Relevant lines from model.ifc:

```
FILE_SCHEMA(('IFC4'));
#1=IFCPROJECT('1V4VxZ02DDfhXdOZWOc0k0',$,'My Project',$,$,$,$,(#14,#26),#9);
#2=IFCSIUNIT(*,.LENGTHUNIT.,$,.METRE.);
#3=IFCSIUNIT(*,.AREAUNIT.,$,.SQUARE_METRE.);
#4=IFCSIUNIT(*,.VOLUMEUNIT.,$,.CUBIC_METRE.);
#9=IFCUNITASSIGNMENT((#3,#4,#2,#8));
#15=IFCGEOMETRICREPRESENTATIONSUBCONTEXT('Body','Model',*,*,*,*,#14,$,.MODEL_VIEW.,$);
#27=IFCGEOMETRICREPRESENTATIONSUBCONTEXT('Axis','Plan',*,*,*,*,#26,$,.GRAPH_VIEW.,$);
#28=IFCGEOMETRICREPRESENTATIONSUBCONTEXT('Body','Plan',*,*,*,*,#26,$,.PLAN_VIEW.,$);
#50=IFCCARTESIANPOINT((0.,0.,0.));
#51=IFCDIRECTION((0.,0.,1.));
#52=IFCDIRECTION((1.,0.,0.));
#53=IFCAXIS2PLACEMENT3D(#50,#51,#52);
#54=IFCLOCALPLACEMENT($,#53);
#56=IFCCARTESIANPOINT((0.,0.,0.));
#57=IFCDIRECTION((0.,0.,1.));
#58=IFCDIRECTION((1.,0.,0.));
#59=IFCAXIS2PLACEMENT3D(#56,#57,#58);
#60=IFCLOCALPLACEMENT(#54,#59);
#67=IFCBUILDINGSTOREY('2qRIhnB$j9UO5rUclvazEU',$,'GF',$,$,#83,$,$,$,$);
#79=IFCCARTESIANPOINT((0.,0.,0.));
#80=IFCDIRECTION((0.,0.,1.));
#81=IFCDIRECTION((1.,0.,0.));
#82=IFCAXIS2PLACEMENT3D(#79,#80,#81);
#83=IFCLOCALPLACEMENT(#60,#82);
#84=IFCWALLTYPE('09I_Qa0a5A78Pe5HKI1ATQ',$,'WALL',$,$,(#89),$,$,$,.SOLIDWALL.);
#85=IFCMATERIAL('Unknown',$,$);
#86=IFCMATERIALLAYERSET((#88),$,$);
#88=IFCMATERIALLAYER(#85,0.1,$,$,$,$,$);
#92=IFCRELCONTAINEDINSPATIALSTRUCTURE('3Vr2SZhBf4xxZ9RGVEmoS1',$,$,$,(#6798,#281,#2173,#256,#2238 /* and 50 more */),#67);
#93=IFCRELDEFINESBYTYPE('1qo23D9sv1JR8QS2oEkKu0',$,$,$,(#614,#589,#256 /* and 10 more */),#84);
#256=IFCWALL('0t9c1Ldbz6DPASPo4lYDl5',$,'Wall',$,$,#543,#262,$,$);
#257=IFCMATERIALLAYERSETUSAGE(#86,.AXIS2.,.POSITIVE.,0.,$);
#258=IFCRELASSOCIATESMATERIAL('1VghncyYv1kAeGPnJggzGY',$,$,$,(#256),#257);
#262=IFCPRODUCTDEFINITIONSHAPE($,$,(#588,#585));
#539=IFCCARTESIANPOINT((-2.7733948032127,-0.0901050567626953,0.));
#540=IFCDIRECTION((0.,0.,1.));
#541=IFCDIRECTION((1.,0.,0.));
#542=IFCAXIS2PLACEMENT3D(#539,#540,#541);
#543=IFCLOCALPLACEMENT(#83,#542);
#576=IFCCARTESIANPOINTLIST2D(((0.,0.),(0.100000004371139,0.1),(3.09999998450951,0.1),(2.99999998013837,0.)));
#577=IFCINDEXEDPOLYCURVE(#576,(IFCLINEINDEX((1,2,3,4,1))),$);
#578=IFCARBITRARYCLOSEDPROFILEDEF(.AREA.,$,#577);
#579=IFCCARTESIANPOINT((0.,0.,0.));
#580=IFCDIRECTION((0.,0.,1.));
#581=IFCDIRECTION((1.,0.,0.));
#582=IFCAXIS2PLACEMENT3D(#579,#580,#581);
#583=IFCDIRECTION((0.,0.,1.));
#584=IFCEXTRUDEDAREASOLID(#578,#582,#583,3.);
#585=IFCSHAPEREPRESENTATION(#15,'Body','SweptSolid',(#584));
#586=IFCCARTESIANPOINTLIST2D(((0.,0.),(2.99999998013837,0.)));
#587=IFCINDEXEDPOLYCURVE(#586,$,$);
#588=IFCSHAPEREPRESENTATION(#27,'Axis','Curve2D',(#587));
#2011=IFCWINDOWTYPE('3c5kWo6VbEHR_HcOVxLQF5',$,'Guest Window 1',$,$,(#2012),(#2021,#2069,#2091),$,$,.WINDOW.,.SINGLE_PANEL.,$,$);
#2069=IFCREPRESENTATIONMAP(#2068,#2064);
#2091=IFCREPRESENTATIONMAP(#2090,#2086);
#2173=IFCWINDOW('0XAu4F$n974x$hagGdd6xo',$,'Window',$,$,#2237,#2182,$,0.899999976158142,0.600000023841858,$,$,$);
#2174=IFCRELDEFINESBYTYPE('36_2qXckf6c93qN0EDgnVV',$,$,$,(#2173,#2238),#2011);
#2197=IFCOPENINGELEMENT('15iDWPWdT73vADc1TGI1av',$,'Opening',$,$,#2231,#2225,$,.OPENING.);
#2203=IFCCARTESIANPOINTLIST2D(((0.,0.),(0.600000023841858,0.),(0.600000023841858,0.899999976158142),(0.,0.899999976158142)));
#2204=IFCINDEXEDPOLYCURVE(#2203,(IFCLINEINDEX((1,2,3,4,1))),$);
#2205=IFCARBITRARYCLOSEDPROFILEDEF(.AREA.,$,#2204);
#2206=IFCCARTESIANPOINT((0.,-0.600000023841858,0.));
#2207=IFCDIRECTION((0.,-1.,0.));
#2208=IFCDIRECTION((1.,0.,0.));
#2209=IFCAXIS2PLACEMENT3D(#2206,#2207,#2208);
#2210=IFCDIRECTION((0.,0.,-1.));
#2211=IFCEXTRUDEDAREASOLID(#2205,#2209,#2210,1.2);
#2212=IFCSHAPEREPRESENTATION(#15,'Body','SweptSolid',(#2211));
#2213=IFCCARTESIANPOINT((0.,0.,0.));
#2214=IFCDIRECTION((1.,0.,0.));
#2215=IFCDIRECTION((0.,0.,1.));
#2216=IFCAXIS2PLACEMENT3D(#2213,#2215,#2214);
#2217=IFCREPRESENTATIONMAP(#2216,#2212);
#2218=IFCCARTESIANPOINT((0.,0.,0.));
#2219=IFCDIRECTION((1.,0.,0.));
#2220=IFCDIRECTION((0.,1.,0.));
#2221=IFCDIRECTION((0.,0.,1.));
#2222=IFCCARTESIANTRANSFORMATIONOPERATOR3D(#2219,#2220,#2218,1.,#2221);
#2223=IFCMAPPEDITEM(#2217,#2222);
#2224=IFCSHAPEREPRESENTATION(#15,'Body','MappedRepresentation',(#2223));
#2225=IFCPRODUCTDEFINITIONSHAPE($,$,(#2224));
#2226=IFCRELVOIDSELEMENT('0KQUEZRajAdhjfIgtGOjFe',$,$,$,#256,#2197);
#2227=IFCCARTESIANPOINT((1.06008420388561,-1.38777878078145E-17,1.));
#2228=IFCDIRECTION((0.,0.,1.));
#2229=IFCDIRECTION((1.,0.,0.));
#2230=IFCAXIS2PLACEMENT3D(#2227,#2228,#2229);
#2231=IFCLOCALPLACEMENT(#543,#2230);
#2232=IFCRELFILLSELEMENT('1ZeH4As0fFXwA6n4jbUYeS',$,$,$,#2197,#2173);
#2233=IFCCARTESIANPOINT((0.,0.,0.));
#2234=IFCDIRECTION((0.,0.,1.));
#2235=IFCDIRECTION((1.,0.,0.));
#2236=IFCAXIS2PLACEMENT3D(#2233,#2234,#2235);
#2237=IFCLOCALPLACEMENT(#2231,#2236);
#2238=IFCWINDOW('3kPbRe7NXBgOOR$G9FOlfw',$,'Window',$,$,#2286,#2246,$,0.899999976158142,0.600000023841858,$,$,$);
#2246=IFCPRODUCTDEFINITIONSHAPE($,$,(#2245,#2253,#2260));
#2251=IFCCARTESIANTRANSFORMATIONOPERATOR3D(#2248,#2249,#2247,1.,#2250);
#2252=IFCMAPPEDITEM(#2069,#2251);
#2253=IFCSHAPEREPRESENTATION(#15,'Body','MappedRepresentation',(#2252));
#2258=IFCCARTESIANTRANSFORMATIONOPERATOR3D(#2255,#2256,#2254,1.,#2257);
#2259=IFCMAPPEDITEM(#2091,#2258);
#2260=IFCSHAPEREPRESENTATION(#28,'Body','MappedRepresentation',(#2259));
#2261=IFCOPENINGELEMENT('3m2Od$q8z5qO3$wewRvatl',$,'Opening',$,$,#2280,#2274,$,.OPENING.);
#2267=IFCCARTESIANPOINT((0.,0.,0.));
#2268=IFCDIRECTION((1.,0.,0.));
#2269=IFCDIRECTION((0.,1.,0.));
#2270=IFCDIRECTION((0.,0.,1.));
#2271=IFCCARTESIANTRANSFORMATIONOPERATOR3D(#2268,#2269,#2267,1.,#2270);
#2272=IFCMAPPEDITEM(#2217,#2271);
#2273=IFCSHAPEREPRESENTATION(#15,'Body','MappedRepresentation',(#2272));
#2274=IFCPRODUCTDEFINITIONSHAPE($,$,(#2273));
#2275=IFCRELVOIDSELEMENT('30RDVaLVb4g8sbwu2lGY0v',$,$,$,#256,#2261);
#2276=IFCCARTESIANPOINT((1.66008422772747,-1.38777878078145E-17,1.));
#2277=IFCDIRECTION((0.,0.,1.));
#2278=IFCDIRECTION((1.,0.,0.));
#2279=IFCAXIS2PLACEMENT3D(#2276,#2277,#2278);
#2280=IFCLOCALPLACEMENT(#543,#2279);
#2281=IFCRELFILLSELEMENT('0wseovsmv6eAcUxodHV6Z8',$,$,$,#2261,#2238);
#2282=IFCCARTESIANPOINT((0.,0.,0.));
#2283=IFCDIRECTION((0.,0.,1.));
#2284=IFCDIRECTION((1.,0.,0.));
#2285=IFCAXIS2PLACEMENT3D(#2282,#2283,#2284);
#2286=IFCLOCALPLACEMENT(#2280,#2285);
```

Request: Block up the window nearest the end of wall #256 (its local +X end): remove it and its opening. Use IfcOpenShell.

```python
import ifcopenshell
import ifcopenshell.api.feature
import ifcopenshell.api.root
import ifcopenshell.geom
import ifcopenshell.util.shape

model = ifcopenshell.open("model.ifc")
settings = ifcopenshell.geom.settings()


def volume(element):
    """Net volume in cubic metres, openings subtracted."""
    shape = ifcopenshell.geom.create_shape(settings, element)
    return ifcopenshell.util.shape.get_volume(shape.geometry)


window = model.by_id(2238)
opening = window.FillsVoids[0].RelatingOpeningElement
wall = opening.VoidsElements[0].RelatingBuildingElement
before = volume(wall)

ifcopenshell.api.root.remove_product(model, product=window)
ifcopenshell.api.feature.remove_feature(model, feature=opening)

after = volume(wall)

print(f"wall volume {before:.3f} -> {after:.3f} m3")

model.write("model_v2.ifc")
```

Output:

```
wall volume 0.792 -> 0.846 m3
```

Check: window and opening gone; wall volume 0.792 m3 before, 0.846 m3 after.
